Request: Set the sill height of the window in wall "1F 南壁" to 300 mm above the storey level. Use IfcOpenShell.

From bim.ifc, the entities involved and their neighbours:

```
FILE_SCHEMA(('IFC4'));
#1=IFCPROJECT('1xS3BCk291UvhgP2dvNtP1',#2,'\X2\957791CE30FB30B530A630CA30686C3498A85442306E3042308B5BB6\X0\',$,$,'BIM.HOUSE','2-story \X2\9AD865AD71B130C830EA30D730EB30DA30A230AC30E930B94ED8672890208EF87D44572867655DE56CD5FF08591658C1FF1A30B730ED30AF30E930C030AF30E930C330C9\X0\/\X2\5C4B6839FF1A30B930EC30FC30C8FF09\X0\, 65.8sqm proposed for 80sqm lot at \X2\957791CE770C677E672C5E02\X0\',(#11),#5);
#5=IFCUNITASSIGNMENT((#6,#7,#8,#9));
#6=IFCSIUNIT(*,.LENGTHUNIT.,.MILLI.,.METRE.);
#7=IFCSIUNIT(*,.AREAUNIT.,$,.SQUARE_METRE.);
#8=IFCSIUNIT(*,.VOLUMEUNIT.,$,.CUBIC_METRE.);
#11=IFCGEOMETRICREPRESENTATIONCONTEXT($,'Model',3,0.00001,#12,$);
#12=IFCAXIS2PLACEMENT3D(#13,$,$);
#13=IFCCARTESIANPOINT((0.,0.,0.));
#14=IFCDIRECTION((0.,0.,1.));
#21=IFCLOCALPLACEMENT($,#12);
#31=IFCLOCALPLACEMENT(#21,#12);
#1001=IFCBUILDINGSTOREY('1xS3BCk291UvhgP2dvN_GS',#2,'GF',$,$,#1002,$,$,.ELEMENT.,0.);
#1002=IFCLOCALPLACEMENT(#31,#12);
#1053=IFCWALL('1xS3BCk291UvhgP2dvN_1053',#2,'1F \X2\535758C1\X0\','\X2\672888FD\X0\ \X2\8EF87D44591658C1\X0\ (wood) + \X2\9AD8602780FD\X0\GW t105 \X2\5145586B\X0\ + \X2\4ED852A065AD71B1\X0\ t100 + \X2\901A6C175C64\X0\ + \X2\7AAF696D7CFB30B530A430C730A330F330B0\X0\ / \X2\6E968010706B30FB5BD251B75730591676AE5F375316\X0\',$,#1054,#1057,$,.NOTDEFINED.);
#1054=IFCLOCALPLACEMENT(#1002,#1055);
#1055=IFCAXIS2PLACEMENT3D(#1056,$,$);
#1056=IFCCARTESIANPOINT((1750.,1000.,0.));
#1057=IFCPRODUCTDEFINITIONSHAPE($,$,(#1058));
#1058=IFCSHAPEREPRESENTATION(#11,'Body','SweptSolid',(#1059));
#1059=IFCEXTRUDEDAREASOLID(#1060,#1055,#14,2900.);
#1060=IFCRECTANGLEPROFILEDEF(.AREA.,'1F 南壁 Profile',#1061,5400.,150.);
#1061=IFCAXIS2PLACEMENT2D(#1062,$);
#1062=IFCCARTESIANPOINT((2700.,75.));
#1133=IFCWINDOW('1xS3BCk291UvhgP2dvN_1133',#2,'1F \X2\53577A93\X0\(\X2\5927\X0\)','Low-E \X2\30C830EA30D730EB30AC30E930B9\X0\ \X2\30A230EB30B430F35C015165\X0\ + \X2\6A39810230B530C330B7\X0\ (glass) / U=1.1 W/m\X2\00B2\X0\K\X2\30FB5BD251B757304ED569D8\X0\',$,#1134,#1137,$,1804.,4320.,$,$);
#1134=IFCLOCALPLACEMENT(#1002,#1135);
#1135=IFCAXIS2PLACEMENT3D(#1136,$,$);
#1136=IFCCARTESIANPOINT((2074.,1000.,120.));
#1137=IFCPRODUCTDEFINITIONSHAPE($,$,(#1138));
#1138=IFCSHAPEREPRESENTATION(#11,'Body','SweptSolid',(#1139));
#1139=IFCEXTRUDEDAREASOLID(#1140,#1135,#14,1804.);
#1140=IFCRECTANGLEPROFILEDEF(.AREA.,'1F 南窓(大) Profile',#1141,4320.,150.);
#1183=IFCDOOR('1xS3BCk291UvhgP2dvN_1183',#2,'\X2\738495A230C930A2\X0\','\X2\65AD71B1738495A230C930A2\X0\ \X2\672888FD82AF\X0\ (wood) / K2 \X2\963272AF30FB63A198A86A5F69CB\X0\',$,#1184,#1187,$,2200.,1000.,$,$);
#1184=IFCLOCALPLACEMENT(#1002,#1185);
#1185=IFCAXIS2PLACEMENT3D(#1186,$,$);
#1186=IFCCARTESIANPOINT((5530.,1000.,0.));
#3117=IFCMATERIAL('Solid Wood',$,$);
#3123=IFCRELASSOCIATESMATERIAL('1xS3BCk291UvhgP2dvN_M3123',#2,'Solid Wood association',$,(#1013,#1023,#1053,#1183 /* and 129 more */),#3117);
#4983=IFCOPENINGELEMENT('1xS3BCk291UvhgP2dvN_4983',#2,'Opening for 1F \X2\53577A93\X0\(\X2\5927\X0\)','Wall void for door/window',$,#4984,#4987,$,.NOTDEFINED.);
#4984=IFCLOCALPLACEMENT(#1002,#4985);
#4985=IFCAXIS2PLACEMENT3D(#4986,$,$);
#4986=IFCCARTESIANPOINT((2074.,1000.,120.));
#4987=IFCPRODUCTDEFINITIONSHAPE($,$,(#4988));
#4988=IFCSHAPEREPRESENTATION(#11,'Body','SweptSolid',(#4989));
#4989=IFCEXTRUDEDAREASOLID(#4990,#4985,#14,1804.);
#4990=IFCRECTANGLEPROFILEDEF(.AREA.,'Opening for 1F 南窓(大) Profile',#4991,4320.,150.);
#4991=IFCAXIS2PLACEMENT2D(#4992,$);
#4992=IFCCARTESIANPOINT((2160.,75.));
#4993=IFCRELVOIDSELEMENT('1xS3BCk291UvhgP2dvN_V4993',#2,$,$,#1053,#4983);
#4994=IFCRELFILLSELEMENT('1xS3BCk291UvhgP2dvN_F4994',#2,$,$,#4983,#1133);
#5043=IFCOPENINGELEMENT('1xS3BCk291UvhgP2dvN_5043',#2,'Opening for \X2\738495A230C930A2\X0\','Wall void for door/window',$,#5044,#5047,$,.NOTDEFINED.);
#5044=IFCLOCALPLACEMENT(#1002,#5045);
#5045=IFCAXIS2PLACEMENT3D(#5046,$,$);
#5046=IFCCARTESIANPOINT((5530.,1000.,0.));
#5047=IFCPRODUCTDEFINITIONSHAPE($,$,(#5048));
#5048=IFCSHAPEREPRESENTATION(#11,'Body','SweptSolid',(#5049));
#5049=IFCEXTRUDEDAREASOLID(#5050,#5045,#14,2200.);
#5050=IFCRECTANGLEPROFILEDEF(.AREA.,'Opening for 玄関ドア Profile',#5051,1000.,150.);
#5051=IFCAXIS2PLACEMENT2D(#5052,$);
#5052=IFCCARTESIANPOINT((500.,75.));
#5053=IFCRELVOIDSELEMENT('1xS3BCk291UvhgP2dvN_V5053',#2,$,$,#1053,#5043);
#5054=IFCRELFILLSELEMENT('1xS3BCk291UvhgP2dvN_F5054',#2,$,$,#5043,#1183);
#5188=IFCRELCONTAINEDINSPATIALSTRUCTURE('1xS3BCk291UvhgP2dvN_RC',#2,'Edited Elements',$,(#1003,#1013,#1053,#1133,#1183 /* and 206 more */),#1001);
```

```python
import numpy as np
import ifcopenshell
import ifcopenshell.api.geometry
import ifcopenshell.geom
import ifcopenshell.util.element
import ifcopenshell.util.placement
import ifcopenshell.util.shape
import ifcopenshell.util.unit

model = ifcopenshell.open("bim.ifc")
unit_scale = ifcopenshell.util.unit.calculate_unit_scale(model)

window = model.by_guid("1xS3BCk291UvhgP2dvN_1133")
opening = window.FillsVoids[0].RelatingOpeningElement
storey = ifcopenshell.util.element.get_container(window, ifc_class="IfcBuildingStorey")
level = ifcopenshell.util.placement.get_local_placement(storey.ObjectPlacement)[2, 3]

# The opening's origin need not be at the sill, so measure its lowest point.
shape = ifcopenshell.geom.create_shape(ifcopenshell.geom.settings(), opening)
bottom = ifcopenshell.util.shape.get_shape_bottom_elevation(shape, shape.geometry) / unit_scale
dz = level + 0.3 / unit_scale - bottom

shift = np.array([0.0, 0.0, dz])
# The window is not placed relative to its opening, so move both.
for product in (opening, window):
    matrix = ifcopenshell.util.placement.get_local_placement(product.ObjectPlacement)
    matrix[:3, 3] += shift
    ifcopenshell.api.geometry.edit_object_placement(model, product=product, matrix=matrix, is_si=False)

print(f"moved by {dz * unit_scale:+.3f} m")

model.write("bim_updated.ifc")
```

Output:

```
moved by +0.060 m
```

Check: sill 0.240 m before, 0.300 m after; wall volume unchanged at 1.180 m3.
